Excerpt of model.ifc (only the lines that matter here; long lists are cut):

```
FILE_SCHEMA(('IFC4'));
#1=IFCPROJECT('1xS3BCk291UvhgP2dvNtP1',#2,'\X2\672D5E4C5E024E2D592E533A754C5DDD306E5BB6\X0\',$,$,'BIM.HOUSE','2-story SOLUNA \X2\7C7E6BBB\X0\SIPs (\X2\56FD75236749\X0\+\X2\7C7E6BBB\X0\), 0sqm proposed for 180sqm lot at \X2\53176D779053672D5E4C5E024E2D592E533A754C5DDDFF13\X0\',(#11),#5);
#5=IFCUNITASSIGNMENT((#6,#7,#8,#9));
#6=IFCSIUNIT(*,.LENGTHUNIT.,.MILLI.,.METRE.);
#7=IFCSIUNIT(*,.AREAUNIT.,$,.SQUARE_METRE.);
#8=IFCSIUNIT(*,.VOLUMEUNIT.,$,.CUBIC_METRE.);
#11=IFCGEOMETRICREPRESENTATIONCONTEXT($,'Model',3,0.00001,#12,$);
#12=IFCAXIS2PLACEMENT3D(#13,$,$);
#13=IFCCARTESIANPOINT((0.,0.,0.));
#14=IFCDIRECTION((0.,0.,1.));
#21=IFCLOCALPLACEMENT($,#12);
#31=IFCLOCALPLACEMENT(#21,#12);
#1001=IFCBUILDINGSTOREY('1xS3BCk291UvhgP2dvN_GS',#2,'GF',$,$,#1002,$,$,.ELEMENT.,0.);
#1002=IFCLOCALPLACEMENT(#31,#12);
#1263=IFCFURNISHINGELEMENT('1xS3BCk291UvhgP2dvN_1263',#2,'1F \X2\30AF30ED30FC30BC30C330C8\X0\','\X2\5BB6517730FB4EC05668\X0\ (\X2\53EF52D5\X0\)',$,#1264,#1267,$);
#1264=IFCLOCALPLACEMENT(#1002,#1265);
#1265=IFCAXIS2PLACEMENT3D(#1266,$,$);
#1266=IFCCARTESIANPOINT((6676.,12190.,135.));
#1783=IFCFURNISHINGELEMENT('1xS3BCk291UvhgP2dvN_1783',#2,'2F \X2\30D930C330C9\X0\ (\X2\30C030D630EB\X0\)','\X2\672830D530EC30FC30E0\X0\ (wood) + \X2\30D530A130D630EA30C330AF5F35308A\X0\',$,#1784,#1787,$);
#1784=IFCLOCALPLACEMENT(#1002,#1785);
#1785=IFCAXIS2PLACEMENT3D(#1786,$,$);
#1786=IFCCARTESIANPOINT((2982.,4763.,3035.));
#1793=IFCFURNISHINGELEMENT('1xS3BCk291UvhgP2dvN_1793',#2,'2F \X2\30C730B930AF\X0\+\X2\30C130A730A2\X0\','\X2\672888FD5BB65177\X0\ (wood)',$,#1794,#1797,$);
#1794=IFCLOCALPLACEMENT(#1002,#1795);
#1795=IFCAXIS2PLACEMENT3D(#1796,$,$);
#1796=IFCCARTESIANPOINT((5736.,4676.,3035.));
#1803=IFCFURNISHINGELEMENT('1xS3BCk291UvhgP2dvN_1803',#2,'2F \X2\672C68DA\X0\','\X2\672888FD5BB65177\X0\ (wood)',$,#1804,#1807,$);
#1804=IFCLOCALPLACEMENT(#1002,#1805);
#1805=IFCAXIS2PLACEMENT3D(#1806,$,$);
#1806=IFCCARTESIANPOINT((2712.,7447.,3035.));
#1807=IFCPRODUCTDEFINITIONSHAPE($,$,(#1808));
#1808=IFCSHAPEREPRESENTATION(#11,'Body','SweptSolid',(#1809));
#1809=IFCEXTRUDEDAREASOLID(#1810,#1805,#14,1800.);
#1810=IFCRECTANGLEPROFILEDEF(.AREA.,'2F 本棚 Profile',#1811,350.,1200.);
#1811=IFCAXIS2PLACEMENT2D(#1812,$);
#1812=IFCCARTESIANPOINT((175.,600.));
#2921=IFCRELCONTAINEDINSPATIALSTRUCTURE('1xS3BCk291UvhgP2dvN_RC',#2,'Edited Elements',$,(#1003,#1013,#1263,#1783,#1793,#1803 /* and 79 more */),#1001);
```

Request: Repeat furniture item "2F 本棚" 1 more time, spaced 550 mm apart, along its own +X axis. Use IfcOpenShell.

```python
import ifcopenshell
import ifcopenshell.api.geometry
import ifcopenshell.api.root
import ifcopenshell.util.element
import ifcopenshell.util.placement
import ifcopenshell.util.unit

model = ifcopenshell.open("model.ifc")
unit_scale = ifcopenshell.util.unit.calculate_unit_scale(model)


def reuse_history(source, copy):
    """copy_class also copies each property set's owner history, people and application; keep the originals."""
    for rel in copy.IsDefinedBy:
        if rel.is_a("IfcRelDefinesByProperties") and (history := rel.RelatingPropertyDefinition.OwnerHistory):
            rel.RelatingPropertyDefinition.OwnerHistory = source.OwnerHistory
            ifcopenshell.util.element.remove_deep2(model, history)


source = model.by_guid("1xS3BCk291UvhgP2dvN_1803")
base = ifcopenshell.util.placement.get_local_placement(source.ObjectPlacement)
step = base[:3, 0] * 0.55 / unit_scale

for i in range(1, 2):
    copy = ifcopenshell.api.root.copy_class(model, product=source)
    copy.Representation = ifcopenshell.util.element.copy_deep(
        model, source.Representation, exclude=["IfcGeometricRepresentationContext", "IfcRepresentationMap"]
    )
    reuse_history(source, copy)
    matrix = base.copy()
    matrix[:3, 3] += i * step
    print("added at", matrix[:3, 3].round(3) + 0.0)
    ifcopenshell.api.geometry.edit_object_placement(model, product=copy, matrix=matrix, is_si=False)

model.write("model_v2.ifc")
```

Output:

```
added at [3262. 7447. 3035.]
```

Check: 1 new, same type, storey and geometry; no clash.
